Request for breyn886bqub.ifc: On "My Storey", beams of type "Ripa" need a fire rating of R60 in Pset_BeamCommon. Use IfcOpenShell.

First a look at what the model holds.

```python
import ifcopenshell
import ifcopenshell.util.element

model = ifcopenshell.open("breyn886bqub.ifc")
print(model.schema)
storey = next(s for s in model.by_type("IfcBuildingStorey") if s.Name == "My Storey")
beams = [e for e in ifcopenshell.util.element.get_decomposition(storey) if e.is_a("IfcBeam")]
seen = {}
for e in beams:
    element_type = ifcopenshell.util.element.get_type(e)
    key = (element_type.Name if element_type != e and element_type else None, ifcopenshell.util.element.get_pset(e, "Pset_BeamCommon", "FireRating"))
    seen[key] = seen.get(key, 0) + 1
for (name, value), count in sorted(seen.items(), key=str):
    print(count, "x", name, "|", value)
```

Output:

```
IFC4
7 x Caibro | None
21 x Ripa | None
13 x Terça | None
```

```python
import ifcopenshell
import ifcopenshell.api.pset
import ifcopenshell.util.element

model = ifcopenshell.open("breyn886bqub.ifc")

storey = next(s for s in model.by_type("IfcBuildingStorey") if s.Name == "My Storey")
beams = [e for e in ifcopenshell.util.element.get_decomposition(storey) if e.is_a("IfcBeam")]

count = 0
for e in beams:
    element_type = ifcopenshell.util.element.get_type(e)
    if element_type in (None, e) or element_type.Name != "Ripa":
        continue
    # add_pset returns the element's existing set when there is one.
    pset = ifcopenshell.api.pset.add_pset(model, product=e, name="Pset_BeamCommon")
    ifcopenshell.api.pset.edit_pset(model, pset=pset, properties={"FireRating": "R60"})
    count += 1

print(count, "beams updated")

model.write("breyn886bqub_updated.ifc")
```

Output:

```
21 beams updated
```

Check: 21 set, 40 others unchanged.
